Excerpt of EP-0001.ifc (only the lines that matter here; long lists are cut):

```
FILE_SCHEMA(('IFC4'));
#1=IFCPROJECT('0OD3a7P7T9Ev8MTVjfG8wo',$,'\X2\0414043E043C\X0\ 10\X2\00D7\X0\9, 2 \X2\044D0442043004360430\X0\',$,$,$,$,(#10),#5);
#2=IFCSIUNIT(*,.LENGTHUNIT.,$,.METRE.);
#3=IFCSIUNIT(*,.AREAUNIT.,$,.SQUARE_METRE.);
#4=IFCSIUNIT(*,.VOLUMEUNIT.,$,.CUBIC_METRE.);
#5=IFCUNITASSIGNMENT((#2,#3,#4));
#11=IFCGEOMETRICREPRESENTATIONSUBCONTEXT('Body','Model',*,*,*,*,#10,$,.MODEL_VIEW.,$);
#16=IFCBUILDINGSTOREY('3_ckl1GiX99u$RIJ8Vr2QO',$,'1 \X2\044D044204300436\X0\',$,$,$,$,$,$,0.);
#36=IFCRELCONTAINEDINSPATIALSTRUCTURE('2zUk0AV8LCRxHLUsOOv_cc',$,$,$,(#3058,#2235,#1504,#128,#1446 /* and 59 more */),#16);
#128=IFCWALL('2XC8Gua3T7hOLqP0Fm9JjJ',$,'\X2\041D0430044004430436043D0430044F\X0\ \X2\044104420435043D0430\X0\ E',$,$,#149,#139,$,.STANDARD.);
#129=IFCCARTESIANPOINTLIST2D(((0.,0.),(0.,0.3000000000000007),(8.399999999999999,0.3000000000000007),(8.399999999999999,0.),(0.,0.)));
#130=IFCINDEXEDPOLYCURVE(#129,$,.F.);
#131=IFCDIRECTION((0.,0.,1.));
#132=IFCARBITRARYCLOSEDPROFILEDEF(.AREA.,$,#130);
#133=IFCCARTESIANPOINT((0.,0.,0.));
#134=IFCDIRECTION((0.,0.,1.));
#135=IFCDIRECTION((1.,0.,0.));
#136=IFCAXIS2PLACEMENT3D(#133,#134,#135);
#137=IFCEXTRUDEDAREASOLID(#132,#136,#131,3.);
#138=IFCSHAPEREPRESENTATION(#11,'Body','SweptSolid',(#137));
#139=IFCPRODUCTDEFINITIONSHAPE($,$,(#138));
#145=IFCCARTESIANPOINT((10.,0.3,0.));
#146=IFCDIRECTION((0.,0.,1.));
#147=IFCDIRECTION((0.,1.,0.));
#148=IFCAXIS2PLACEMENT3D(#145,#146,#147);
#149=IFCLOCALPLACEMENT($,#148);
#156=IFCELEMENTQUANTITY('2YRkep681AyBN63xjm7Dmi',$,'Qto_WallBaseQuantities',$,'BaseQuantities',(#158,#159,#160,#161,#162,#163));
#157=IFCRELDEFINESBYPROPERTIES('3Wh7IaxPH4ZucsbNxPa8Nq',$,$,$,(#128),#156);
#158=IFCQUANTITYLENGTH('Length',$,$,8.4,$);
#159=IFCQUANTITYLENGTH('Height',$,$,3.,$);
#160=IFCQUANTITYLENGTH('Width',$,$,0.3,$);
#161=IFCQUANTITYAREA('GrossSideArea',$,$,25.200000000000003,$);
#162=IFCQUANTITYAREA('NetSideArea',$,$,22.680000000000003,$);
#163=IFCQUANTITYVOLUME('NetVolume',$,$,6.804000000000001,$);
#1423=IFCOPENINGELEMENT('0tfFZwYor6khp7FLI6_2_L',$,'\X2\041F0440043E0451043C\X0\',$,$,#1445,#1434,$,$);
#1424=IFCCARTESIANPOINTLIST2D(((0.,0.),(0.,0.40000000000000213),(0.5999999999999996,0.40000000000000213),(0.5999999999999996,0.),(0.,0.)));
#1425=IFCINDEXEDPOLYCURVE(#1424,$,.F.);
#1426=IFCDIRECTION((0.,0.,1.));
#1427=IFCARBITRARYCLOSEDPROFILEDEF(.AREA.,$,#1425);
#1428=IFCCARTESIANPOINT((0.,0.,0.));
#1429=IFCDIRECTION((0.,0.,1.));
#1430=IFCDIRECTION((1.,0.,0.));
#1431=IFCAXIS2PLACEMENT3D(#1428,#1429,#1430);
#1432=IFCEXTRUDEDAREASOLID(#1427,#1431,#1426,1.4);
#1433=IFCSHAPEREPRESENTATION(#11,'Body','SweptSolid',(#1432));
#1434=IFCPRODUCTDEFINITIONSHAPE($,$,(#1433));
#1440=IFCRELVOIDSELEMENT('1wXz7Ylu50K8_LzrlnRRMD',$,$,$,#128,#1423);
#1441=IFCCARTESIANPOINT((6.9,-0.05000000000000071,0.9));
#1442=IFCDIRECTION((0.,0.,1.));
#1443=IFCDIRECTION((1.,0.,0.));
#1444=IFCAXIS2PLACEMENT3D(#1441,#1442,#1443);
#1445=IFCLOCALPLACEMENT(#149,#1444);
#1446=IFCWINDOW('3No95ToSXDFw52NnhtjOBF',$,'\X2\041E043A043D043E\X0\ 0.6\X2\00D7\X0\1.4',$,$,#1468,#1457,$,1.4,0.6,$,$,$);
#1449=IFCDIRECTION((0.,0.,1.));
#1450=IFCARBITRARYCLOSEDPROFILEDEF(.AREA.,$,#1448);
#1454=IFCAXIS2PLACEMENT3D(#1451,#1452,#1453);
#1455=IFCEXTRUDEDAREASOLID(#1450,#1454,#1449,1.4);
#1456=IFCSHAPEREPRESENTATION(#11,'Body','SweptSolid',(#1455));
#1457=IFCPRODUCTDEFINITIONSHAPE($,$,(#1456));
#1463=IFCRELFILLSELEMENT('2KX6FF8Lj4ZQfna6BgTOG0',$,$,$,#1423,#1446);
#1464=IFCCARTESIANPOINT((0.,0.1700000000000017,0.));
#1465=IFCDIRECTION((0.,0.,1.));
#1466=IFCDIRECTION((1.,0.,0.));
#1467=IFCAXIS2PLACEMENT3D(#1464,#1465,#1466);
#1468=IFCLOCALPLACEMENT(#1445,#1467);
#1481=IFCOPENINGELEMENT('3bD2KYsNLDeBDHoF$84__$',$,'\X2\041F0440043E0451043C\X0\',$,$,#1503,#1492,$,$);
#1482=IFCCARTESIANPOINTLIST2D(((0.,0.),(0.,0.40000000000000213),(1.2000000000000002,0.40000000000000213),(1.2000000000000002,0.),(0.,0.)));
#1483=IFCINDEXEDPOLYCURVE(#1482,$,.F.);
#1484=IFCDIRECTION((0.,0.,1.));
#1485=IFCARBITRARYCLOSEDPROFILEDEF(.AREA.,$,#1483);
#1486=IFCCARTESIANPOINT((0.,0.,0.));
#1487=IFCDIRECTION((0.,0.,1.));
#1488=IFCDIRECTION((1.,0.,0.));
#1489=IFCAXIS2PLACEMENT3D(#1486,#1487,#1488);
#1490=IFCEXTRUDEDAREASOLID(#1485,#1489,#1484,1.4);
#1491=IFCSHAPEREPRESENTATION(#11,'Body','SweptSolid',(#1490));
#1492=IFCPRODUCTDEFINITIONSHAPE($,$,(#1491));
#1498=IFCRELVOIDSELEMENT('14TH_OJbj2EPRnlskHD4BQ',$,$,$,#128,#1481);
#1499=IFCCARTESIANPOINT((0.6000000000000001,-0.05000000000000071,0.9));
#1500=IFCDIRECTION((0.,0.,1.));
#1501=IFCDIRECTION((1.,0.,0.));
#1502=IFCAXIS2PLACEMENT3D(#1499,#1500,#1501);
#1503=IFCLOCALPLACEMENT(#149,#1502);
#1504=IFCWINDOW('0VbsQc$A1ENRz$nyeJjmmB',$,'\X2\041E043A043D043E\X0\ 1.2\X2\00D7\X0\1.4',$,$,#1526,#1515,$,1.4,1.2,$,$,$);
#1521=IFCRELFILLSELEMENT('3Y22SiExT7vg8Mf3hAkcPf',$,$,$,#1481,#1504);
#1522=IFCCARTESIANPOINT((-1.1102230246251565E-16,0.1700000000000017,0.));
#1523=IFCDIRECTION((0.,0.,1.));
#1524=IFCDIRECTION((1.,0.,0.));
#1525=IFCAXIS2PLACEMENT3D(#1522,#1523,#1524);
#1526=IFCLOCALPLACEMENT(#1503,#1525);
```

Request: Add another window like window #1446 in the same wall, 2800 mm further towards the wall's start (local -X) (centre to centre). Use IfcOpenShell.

```python
import ifcopenshell
import ifcopenshell.api.feature
import ifcopenshell.api.geometry
import ifcopenshell.api.pset
import ifcopenshell.api.root
import ifcopenshell.geom
import ifcopenshell.util.element
import ifcopenshell.util.placement
import ifcopenshell.util.shape
import ifcopenshell.util.unit

model = ifcopenshell.open("EP-0001.ifc")
unit_scale = ifcopenshell.util.unit.calculate_unit_scale(model)
area_scale = ifcopenshell.util.unit.calculate_unit_scale(model, "AREAUNIT")
volume_scale = ifcopenshell.util.unit.calculate_unit_scale(model, "VOLUMEUNIT")
settings = ifcopenshell.geom.settings()


def volume(element):
    """Net volume in cubic metres, openings subtracted."""
    shape = ifcopenshell.geom.create_shape(settings, element)
    return ifcopenshell.util.shape.get_volume(shape.geometry)


window = model.by_id(1446)
opening = window.FillsVoids[0].RelatingOpeningElement
wall = opening.VoidsElements[0].RelatingBuildingElement
before = volume(wall)
shift = ifcopenshell.util.placement.get_local_placement(wall.ObjectPlacement)[:3, 0] * -2.8 / unit_scale

# copy_class copies the void relationship, type, container and properties, but no geometry.
new_opening = ifcopenshell.api.root.copy_class(model, product=opening)
new_opening.Representation = ifcopenshell.util.element.copy_deep(
    model, opening.Representation, exclude=["IfcGeometricRepresentationContext", "IfcRepresentationMap"]
)
new_window = ifcopenshell.api.root.copy_class(model, product=window)
new_window.Representation = ifcopenshell.util.element.copy_deep(
    model, window.Representation, exclude=["IfcGeometricRepresentationContext", "IfcRepresentationMap"]
)
ifcopenshell.api.feature.add_filling(model, opening=new_opening, element=new_window)

for old, new in ((opening, new_opening), (window, new_window)):
    matrix = ifcopenshell.util.placement.get_local_placement(old.ObjectPlacement)
    matrix[:3, 3] += shift
    ifcopenshell.api.geometry.edit_object_placement(model, product=new, matrix=matrix, is_si=False)

after = volume(wall)
thickness = 0.3  # wall thickness in metres

# Update the wall's stored quantities.
qto = model.by_id(ifcopenshell.util.element.get_pset(wall, "Qto_WallBaseQuantities", should_inherit=False)["id"])
ifcopenshell.api.pset.edit_qto(model, qto=qto, properties={
    "NetSideArea": after / thickness / area_scale,
    "NetVolume": after / volume_scale,
})

print(f"wall volume {before:.3f} -> {after:.3f} m3")

model.write("EP-0001_edited.ifc")
```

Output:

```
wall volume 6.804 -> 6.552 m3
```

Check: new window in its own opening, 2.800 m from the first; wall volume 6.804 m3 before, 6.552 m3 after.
